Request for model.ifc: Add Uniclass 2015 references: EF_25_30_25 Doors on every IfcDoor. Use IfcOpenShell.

First a look at what the model holds.

```python
import ifcopenshell

model = ifcopenshell.open("model.ifc")
print(model.schema)
print("classifications:", [c.Name for c in model.by_type("IfcClassification")])
for ifc_class in ("IfcDoor", "IfcRoof", "IfcStair", "IfcWall", "IfcWindow"):
    print(ifc_class, len(model.by_type(ifc_class)))
```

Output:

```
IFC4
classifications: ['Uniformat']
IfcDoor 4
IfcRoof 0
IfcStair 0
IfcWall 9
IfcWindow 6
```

```python
import ifcopenshell
import ifcopenshell.api.classification

model = ifcopenshell.open("model.ifc")

system = ifcopenshell.api.classification.add_classification(model, classification="Uniclass 2015")

codes = {
    "IfcDoor": ("EF_25_30_25", "Doors"),
}
for ifc_class, (code, name) in codes.items():
    products = model.by_type(ifc_class)
    ifcopenshell.api.classification.add_reference(
        model, products=products, classification=system, identification=code, name=name
    )
    print(code, len(products))

model.write("model-out.ifc")
```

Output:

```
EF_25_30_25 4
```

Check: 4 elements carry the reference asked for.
